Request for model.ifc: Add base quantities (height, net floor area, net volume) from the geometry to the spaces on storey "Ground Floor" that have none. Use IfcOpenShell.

First a look at what the model holds.

```python
import ifcopenshell
import ifcopenshell.util.element
import ifcopenshell.util.unit

model = ifcopenshell.open("model.ifc")
print(model.schema)
for unit_type in ("LENGTHUNIT", "AREAUNIT", "VOLUMEUNIT"):
    print(unit_type, ifcopenshell.util.unit.calculate_unit_scale(model, unit_type))
storey = next(s for s in model.by_type("IfcBuildingStorey") if s.Name == "Ground Floor")
spaces = [e for e in ifcopenshell.util.element.get_decomposition(storey) if e.is_a("IfcSpace")]
for e in sorted(spaces, key=lambda e: e.id()):
    print(e.id(), e.is_a(), e.Name, list(ifcopenshell.util.element.get_psets(e, qtos_only=True)), sep=" | ")
```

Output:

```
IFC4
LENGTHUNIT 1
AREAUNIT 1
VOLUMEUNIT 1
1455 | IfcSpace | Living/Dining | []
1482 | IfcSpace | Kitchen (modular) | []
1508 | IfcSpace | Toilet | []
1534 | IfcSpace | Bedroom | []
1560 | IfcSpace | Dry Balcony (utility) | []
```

```python
import ifcopenshell
import ifcopenshell.api.pset
import ifcopenshell.geom
import ifcopenshell.util.element
import ifcopenshell.util.shape
import ifcopenshell.util.unit

model = ifcopenshell.open("model.ifc")
unit_scale = ifcopenshell.util.unit.calculate_unit_scale(model)
area_scale = ifcopenshell.util.unit.calculate_unit_scale(model, "AREAUNIT")
volume_scale = ifcopenshell.util.unit.calculate_unit_scale(model, "VOLUMEUNIT")
settings = ifcopenshell.geom.settings()

storey = next(s for s in model.by_type("IfcBuildingStorey") if s.Name == "Ground Floor")
spaces = [e for e in ifcopenshell.util.element.get_decomposition(storey) if e.is_a("IfcSpace")]

for e in sorted(spaces, key=lambda e: e.id()):
    if ifcopenshell.util.element.get_psets(e, qtos_only=True, should_inherit=False):
        continue
    # Geometry comes back in metres, in the element's own axes.
    shape = ifcopenshell.geom.create_shape(settings, e)
    values = {
        "Height": ifcopenshell.util.shape.get_z(shape.geometry) / unit_scale,
        "NetFloorArea": ifcopenshell.util.shape.get_footprint_area(shape.geometry) / area_scale,
        "NetVolume": ifcopenshell.util.shape.get_volume(shape.geometry) / volume_scale,
    }
    qto = ifcopenshell.api.pset.add_qto(model, product=e, name="Qto_SpaceBaseQuantities")
    ifcopenshell.api.pset.edit_qto(model, qto=qto, properties=values)
    print(e.id(), {k: round(v, 3) for k, v in values.items()})

model.write("model_updated.ifc")
```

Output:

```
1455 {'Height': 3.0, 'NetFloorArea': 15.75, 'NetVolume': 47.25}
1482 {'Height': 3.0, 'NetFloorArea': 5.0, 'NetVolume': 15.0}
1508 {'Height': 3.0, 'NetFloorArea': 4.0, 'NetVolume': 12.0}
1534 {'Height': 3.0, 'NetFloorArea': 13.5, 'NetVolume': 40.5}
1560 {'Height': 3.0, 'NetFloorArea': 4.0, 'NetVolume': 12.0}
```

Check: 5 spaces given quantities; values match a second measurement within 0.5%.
